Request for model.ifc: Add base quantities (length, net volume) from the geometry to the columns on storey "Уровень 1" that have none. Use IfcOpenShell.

First a look at what the model holds.

```python
import ifcopenshell
import ifcopenshell.util.element
import ifcopenshell.util.unit

model = ifcopenshell.open("model.ifc")
print(model.schema)
for unit_type in ("LENGTHUNIT", "AREAUNIT", "VOLUMEUNIT"):
    print(unit_type, ifcopenshell.util.unit.calculate_unit_scale(model, unit_type))
storey = next(s for s in model.by_type("IfcBuildingStorey") if s.Name == "Уровень 1")
columns = [e for e in ifcopenshell.util.element.get_decomposition(storey) if e.is_a("IfcColumn")]
for e in sorted(columns, key=lambda e: e.id()):
    print(e.id(), e.is_a(), e.Name, list(ifcopenshell.util.element.get_psets(e, qtos_only=True)), sep=" | ")
```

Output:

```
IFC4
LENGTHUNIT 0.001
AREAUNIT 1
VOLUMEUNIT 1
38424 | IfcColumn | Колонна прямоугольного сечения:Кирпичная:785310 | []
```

```python
import ifcopenshell
import ifcopenshell.api.pset
import ifcopenshell.geom
import ifcopenshell.util.element
import ifcopenshell.util.shape
import ifcopenshell.util.unit

model = ifcopenshell.open("model.ifc")
unit_scale = ifcopenshell.util.unit.calculate_unit_scale(model)
volume_scale = ifcopenshell.util.unit.calculate_unit_scale(model, "VOLUMEUNIT")
settings = ifcopenshell.geom.settings()

storey = next(s for s in model.by_type("IfcBuildingStorey") if s.Name == "Уровень 1")
columns = [e for e in ifcopenshell.util.element.get_decomposition(storey) if e.is_a("IfcColumn")]

for e in sorted(columns, key=lambda e: e.id()):
    if ifcopenshell.util.element.get_psets(e, qtos_only=True, should_inherit=False):
        continue
    # Geometry comes back in metres, in the element's own axes.
    shape = ifcopenshell.geom.create_shape(settings, e)
    values = {
        "Length": ifcopenshell.util.shape.get_z(shape.geometry) / unit_scale,
        "NetVolume": ifcopenshell.util.shape.get_volume(shape.geometry) / volume_scale,
    }
    qto = ifcopenshell.api.pset.add_qto(model, product=e, name="Qto_ColumnBaseQuantities")
    ifcopenshell.api.pset.edit_qto(model, qto=qto, properties=values)
    print(e.id(), {k: round(v, 3) for k, v in values.items()})

model.write("model_v2.ifc")
```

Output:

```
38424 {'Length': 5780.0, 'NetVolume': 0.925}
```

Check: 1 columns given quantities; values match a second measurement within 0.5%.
